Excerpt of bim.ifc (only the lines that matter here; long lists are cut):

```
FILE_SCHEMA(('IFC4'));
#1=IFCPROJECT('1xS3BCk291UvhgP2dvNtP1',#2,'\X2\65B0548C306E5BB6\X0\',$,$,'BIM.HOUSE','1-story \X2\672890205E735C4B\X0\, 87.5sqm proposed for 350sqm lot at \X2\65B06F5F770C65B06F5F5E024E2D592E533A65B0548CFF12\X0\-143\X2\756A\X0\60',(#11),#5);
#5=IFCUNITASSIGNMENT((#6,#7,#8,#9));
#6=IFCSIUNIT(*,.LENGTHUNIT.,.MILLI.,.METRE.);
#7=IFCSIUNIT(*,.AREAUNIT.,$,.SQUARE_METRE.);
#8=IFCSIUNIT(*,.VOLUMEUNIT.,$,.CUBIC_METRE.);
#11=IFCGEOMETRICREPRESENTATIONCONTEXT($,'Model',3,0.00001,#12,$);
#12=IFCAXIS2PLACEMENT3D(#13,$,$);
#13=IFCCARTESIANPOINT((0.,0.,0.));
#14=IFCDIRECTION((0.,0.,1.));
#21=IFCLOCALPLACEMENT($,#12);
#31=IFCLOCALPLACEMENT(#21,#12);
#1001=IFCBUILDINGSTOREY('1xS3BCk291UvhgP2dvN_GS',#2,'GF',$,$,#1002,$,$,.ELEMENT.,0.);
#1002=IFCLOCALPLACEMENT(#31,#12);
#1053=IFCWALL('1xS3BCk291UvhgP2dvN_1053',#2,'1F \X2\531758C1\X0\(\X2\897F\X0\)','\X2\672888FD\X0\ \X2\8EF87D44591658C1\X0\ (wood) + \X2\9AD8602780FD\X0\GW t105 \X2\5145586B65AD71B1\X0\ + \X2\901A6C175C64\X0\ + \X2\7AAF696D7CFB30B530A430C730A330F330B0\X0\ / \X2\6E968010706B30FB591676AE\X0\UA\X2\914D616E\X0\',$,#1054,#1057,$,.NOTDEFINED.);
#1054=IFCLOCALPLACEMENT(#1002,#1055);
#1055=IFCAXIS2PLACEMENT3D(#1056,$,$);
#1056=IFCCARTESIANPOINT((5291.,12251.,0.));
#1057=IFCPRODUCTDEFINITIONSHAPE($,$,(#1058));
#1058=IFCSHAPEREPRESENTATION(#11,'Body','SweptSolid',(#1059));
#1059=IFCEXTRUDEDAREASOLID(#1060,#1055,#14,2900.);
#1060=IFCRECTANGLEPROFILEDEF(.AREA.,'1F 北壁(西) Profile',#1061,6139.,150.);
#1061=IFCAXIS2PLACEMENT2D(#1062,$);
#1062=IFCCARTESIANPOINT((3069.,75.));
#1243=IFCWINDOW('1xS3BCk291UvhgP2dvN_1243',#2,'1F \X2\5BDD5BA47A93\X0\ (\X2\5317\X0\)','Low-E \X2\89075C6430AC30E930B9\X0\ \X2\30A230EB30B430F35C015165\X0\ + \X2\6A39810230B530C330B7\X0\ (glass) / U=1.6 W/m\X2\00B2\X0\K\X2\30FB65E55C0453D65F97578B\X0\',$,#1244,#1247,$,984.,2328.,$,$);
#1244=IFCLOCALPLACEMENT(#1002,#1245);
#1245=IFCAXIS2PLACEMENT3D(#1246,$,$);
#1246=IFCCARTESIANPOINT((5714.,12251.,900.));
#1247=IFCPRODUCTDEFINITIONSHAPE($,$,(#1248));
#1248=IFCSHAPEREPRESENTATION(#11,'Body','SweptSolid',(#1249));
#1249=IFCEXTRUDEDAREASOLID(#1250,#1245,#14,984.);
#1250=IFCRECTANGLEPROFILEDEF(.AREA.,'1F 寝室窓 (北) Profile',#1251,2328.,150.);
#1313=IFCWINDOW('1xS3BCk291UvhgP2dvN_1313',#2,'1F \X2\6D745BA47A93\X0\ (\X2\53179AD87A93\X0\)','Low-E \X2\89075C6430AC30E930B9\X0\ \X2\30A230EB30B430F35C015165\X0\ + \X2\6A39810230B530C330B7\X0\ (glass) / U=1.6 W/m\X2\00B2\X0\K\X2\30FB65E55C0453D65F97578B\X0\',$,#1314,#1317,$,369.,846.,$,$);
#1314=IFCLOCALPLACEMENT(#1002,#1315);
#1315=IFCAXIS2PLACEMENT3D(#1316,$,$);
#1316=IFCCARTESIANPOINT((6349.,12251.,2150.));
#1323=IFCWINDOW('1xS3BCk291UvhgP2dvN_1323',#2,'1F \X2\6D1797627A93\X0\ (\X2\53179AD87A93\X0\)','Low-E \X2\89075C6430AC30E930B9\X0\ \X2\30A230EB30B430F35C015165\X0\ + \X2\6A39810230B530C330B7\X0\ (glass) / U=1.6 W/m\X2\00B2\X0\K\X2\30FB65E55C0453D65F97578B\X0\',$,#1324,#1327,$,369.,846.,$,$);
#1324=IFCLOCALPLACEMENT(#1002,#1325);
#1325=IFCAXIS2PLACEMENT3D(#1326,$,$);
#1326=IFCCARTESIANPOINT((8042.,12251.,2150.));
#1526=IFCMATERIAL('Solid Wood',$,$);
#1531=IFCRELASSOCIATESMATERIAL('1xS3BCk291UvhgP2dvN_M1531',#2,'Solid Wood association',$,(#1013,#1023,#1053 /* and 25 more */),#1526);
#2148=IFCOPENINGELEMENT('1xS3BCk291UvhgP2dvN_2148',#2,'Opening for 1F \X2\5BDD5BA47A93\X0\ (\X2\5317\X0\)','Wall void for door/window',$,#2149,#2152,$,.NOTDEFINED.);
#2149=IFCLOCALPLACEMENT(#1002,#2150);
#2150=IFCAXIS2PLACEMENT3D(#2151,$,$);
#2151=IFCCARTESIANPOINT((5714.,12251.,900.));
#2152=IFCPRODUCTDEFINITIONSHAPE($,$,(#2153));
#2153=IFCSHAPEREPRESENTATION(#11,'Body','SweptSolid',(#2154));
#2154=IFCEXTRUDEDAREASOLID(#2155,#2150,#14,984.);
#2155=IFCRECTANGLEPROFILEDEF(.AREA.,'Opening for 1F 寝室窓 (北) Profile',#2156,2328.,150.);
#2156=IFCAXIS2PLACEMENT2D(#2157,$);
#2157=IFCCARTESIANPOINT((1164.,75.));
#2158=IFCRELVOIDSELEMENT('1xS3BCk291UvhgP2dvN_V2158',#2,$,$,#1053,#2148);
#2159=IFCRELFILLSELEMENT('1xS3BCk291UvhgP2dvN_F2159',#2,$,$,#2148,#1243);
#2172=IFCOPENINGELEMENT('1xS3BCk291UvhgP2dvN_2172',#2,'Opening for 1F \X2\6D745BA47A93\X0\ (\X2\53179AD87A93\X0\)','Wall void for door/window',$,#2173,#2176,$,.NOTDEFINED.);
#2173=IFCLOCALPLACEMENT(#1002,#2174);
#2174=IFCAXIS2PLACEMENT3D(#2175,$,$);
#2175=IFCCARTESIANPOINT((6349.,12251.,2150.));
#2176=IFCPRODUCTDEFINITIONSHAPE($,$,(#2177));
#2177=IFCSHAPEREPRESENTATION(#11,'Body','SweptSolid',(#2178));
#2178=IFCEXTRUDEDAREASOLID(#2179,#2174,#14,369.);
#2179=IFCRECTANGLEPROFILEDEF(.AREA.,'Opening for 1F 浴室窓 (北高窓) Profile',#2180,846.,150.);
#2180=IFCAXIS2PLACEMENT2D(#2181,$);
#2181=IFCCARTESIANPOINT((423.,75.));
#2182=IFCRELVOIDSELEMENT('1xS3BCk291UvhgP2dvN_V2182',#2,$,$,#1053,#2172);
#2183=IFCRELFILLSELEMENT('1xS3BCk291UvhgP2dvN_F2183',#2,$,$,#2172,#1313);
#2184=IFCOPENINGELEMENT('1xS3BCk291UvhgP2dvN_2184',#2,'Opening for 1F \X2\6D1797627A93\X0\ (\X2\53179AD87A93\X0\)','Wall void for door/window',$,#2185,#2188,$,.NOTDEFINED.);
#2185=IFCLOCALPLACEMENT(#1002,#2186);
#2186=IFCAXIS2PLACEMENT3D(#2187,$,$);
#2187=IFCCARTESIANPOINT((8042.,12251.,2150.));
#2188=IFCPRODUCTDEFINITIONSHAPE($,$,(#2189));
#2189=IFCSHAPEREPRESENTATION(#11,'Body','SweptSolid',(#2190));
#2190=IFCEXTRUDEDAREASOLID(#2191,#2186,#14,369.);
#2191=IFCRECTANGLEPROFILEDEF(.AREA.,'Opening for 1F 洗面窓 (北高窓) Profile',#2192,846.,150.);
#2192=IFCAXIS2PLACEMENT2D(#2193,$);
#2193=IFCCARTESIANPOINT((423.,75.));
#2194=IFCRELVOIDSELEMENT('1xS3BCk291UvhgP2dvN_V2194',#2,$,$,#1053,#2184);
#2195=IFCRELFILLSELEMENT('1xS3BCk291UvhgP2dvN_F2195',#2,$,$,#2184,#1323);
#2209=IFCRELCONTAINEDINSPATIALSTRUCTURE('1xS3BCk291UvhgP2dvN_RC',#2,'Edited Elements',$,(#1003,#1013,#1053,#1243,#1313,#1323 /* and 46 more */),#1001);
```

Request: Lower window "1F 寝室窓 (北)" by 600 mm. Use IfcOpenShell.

```python
import numpy as np
import ifcopenshell
import ifcopenshell.api.geometry
import ifcopenshell.util.placement
import ifcopenshell.util.unit

model = ifcopenshell.open("bim.ifc")
unit_scale = ifcopenshell.util.unit.calculate_unit_scale(model)

window = model.by_guid("1xS3BCk291UvhgP2dvN_1243")
opening = window.FillsVoids[0].RelatingOpeningElement
dz = -0.6 / unit_scale

shift = np.array([0.0, 0.0, dz])
# The window is not placed relative to its opening, so move both.
for product in (opening, window):
    matrix = ifcopenshell.util.placement.get_local_placement(product.ObjectPlacement)
    matrix[:3, 3] += shift
    ifcopenshell.api.geometry.edit_object_placement(model, product=product, matrix=matrix, is_si=False)

print(f"moved by {dz * unit_scale:+.3f} m")

model.write("bim-out.ifc")
```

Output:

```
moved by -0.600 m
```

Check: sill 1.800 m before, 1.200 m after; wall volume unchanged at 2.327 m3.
